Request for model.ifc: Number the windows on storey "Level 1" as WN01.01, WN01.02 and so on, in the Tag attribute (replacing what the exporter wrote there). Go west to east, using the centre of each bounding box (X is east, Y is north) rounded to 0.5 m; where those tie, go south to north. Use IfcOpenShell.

First a look at what the model holds.

```python
import ifcopenshell
import ifcopenshell.util.element
import ifcopenshell.util.placement

model = ifcopenshell.open("model.ifc")
print(model.schema)
storey = next(s for s in model.by_type("IfcBuildingStorey") if s.Name == "Level 1")
windows = [e for e in ifcopenshell.util.element.get_decomposition(storey) if e.is_a("IfcWindow")]
for e in sorted(windows, key=lambda e: e.id()):
    origin = ifcopenshell.util.placement.get_local_placement(e.ObjectPlacement)[:3, 3]
    print(e.id(), e.Tag, e.Name, origin.round(2) + 0.0, sep=" | ")
```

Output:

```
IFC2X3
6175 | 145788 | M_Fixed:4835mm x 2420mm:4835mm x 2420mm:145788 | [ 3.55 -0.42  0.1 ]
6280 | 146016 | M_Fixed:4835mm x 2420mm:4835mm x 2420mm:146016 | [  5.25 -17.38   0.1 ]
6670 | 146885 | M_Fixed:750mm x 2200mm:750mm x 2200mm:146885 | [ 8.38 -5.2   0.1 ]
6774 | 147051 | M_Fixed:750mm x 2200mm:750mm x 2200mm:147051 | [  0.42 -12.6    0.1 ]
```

```python
import ifcopenshell
import ifcopenshell.geom
import ifcopenshell.util.element
import ifcopenshell.util.shape

model = ifcopenshell.open("model.ifc")
settings = ifcopenshell.geom.settings()
settings.set("use-world-coords", True)


def centre(element):
    shape = ifcopenshell.geom.create_shape(settings, element)
    return ifcopenshell.util.shape.get_bbox_centroid(shape.geometry)


storey = next(s for s in model.by_type("IfcBuildingStorey") if s.Name == "Level 1")
windows = [e for e in ifcopenshell.util.element.get_decomposition(storey) if e.is_a("IfcWindow")]

# Insertion points can sit at a corner or the storey origin, so sort by the geometry (in metres).
centres = {e: centre(e) for e in windows}
windows.sort(key=lambda e: (round(centres[e][0] / 0.5), centres[e][1]))

for i, e in enumerate(windows, start=1):
    number = f"WN01.{i:02d}"
    e.Tag = number
    print(e.id(), number)

model.write("model_updated.ifc")
```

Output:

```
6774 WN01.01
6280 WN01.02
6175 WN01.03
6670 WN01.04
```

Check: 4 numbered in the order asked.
